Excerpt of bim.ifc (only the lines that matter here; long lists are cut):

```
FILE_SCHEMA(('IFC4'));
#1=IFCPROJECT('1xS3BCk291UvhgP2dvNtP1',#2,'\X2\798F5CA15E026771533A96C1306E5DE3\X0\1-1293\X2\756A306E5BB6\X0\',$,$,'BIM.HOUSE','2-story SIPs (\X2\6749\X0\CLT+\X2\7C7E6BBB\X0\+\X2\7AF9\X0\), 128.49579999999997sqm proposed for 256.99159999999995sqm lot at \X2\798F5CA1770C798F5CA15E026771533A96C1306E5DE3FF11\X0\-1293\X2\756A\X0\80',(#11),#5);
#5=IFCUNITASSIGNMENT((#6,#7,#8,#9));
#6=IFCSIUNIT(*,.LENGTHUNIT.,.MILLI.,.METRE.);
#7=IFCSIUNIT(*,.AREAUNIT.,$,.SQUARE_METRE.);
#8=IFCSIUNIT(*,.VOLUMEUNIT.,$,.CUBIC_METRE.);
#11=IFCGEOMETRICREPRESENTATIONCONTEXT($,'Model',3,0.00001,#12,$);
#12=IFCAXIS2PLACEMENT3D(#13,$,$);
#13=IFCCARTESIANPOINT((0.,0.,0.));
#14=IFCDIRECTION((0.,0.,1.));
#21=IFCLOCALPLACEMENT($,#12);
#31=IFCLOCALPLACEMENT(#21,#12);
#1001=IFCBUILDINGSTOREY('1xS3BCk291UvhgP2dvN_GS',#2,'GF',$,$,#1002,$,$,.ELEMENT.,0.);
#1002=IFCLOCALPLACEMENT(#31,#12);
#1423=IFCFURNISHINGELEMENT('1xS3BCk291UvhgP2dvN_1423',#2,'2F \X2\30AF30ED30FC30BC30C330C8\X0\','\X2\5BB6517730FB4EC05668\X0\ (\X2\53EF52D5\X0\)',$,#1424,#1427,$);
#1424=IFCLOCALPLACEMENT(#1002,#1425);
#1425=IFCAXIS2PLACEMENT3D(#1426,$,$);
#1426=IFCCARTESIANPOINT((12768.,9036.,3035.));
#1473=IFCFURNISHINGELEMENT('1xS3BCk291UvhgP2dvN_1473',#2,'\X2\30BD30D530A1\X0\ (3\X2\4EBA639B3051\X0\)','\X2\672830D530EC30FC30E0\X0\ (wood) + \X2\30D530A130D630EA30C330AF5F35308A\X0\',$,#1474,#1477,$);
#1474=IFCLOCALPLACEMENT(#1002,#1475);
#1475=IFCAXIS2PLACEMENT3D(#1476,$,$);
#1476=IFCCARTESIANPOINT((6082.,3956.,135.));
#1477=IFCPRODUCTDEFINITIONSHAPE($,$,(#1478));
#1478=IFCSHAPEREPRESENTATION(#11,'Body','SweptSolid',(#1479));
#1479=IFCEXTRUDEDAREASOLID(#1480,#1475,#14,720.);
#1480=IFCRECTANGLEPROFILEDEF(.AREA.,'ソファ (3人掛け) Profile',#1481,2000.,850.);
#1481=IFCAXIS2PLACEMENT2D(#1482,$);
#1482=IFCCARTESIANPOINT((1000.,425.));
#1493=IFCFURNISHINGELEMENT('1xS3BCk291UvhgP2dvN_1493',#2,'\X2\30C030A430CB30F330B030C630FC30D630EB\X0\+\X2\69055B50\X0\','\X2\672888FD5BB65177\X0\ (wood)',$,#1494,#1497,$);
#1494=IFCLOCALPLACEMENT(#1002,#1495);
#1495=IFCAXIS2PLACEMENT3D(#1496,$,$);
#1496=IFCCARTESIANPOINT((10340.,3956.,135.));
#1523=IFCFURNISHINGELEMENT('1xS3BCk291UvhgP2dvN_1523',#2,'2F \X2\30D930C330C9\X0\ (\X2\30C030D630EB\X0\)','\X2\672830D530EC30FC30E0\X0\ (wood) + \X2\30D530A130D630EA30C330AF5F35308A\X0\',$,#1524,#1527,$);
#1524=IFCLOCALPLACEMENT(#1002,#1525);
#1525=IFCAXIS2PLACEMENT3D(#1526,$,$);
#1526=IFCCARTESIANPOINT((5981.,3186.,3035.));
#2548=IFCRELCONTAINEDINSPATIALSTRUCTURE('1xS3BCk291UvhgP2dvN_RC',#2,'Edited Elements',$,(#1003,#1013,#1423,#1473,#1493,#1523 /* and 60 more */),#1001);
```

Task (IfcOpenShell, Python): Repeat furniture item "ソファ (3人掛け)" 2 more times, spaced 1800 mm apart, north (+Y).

```python
import numpy as np
import ifcopenshell
import ifcopenshell.api.geometry
import ifcopenshell.api.root
import ifcopenshell.util.element
import ifcopenshell.util.placement

model = ifcopenshell.open("bim.ifc")


def reuse_history(source, copy):
    """copy_class also copies each property set's owner history, people and application; keep the originals."""
    for rel in copy.IsDefinedBy:
        if rel.is_a("IfcRelDefinesByProperties") and (history := rel.RelatingPropertyDefinition.OwnerHistory):
            rel.RelatingPropertyDefinition.OwnerHistory = source.OwnerHistory
            ifcopenshell.util.element.remove_deep2(model, history)


source = model.by_guid("1xS3BCk291UvhgP2dvN_1473")
base = ifcopenshell.util.placement.get_local_placement(source.ObjectPlacement)
step = np.array([0.0, 1.0, 0.0]) * 1800.0

for i in range(1, 3):
    copy = ifcopenshell.api.root.copy_class(model, product=source)
    copy.Representation = ifcopenshell.util.element.copy_deep(
        model, source.Representation, exclude=["IfcGeometricRepresentationContext", "IfcRepresentationMap"]
    )
    reuse_history(source, copy)
    matrix = base.copy()
    matrix[:3, 3] += i * step
    print("added at", matrix[:3, 3].round(3) + 0.0)
    ifcopenshell.api.geometry.edit_object_placement(model, product=copy, matrix=matrix, is_si=False)

model.write("bim_v2.ifc")
```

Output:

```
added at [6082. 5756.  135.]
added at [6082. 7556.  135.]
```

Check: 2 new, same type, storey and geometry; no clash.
